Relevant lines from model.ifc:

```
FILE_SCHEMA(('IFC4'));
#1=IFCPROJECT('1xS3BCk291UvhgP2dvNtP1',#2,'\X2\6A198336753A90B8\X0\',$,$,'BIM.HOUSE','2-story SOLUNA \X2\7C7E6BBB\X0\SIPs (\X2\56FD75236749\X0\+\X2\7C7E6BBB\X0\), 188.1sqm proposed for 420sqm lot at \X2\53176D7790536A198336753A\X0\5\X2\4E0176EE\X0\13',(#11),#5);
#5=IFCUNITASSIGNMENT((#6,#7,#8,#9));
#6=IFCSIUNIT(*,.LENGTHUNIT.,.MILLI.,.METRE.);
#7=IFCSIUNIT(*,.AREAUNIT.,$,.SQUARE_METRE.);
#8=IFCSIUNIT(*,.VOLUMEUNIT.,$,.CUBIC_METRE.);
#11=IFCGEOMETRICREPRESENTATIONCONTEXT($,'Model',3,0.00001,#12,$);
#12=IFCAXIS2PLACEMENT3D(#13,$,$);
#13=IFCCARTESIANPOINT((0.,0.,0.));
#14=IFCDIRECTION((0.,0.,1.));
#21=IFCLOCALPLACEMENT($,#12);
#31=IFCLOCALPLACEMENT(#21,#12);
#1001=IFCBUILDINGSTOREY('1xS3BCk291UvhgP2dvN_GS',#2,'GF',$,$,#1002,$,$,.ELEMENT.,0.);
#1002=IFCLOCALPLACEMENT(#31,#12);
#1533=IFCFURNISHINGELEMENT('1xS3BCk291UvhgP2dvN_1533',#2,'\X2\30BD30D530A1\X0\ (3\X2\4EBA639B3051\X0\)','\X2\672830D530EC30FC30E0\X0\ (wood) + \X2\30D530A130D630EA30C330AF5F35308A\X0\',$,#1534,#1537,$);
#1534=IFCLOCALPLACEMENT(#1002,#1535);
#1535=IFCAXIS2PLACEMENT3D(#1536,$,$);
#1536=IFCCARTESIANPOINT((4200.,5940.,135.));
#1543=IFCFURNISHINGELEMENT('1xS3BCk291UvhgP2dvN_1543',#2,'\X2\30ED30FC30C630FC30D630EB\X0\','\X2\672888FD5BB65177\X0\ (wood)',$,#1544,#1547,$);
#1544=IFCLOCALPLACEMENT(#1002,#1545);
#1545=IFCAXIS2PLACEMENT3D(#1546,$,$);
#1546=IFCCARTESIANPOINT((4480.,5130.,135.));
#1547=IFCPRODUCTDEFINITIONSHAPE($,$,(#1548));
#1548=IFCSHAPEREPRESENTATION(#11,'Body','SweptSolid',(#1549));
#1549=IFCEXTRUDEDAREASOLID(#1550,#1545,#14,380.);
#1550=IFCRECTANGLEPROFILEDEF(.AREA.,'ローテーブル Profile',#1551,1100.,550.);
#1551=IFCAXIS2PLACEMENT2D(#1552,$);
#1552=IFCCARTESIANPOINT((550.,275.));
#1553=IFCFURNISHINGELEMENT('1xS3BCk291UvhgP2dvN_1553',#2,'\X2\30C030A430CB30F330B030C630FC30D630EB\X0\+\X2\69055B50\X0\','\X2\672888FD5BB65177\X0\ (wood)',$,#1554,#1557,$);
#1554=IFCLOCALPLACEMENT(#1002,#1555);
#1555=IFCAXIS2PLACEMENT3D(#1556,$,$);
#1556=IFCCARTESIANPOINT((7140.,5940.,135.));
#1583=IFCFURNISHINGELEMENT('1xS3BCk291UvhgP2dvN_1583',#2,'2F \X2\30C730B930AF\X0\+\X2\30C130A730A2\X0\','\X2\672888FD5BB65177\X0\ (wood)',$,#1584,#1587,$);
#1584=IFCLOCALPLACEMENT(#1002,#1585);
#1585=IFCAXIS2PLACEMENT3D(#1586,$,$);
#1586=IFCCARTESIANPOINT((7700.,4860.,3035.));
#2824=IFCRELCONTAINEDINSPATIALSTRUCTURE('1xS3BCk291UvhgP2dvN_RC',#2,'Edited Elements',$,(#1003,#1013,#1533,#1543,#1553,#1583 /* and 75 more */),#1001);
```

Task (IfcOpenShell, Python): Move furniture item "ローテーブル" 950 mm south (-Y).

```python
import ifcopenshell
import ifcopenshell.api.geometry
import ifcopenshell.util.placement

model = ifcopenshell.open("model.ifc")

item = model.by_guid("1xS3BCk291UvhgP2dvN_1543")
matrix = ifcopenshell.util.placement.get_local_placement(item.ObjectPlacement)
matrix[1, 3] -= 950.0
ifcopenshell.api.geometry.edit_object_placement(model, product=item, matrix=matrix, is_si=False)

print(ifcopenshell.util.placement.get_local_placement(item.ObjectPlacement).round(3) + 0.0)

model.write("model-out.ifc")
```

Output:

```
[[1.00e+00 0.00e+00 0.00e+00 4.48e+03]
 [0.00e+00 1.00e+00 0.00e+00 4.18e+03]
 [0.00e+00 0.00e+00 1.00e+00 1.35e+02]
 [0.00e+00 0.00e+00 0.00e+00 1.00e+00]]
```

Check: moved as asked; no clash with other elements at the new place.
